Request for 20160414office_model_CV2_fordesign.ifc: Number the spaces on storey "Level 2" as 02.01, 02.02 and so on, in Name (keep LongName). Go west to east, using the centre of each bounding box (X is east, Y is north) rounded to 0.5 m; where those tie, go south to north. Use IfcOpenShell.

First a look at what the model holds.

```python
import ifcopenshell
import ifcopenshell.util.element
import ifcopenshell.util.placement

model = ifcopenshell.open("20160414office_model_CV2_fordesign.ifc")
print(model.schema)
storey = next(s for s in model.by_type("IfcBuildingStorey") if s.Name == "Level 2")
spaces = [e for e in ifcopenshell.util.element.get_decomposition(storey) if e.is_a("IfcSpace")]
for e in sorted(spaces, key=lambda e: e.id()):
    origin = ifcopenshell.util.placement.get_local_placement(e.ObjectPlacement)[:3, 3]
    print(e.id(), e.Name, e.LongName, origin.round(2) + 0.0, sep=" | ")
```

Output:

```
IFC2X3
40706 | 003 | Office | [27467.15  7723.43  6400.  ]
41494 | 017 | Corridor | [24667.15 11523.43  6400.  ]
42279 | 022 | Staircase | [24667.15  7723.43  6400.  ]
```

```python
import ifcopenshell
import ifcopenshell.geom
import ifcopenshell.util.element
import ifcopenshell.util.shape

model = ifcopenshell.open("20160414office_model_CV2_fordesign.ifc")
settings = ifcopenshell.geom.settings()
settings.set("use-world-coords", True)


def centre(element):
    shape = ifcopenshell.geom.create_shape(settings, element)
    return ifcopenshell.util.shape.get_bbox_centroid(shape.geometry)


storey = next(s for s in model.by_type("IfcBuildingStorey") if s.Name == "Level 2")
spaces = [e for e in ifcopenshell.util.element.get_decomposition(storey) if e.is_a("IfcSpace")]

# Insertion points can sit at a corner or the storey origin, so sort by the geometry (in metres).
centres = {e: centre(e) for e in spaces}
spaces.sort(key=lambda e: (round(centres[e][0] / 0.5), centres[e][1]))

for i, e in enumerate(spaces, start=1):
    number = f"02.{i:02d}"
    e.Name = number
    print(e.id(), number)

model.write("20160414office_model_CV2_fordesign_v2.ifc")
```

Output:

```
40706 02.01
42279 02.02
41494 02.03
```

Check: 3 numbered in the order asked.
